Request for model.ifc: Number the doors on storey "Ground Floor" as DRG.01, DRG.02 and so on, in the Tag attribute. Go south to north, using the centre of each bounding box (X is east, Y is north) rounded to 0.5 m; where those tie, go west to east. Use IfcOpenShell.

First a look at what the model holds.

```python
import ifcopenshell
import ifcopenshell.util.element
import ifcopenshell.util.placement

model = ifcopenshell.open("model.ifc")
print(model.schema)
storey = next(s for s in model.by_type("IfcBuildingStorey") if s.Name == "Ground Floor")
doors = [e for e in ifcopenshell.util.element.get_decomposition(storey) if e.is_a("IfcDoor")]
for e in sorted(doors, key=lambda e: e.id()):
    origin = ifcopenshell.util.placement.get_local_placement(e.ObjectPlacement)[:3, 3]
    print(e.id(), e.Tag, e.Name, origin.round(2) + 0.0, sep=" | ")
```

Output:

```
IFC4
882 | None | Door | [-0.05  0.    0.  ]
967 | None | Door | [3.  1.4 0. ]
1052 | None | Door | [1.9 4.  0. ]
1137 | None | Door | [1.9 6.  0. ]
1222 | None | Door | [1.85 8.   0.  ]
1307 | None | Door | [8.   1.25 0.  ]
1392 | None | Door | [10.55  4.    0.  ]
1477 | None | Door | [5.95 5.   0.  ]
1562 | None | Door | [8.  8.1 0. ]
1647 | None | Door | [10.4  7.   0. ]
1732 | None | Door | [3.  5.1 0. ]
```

```python
import ifcopenshell
import ifcopenshell.geom
import ifcopenshell.util.element
import ifcopenshell.util.shape

model = ifcopenshell.open("model.ifc")
settings = ifcopenshell.geom.settings()
settings.set("use-world-coords", True)


def centre(element):
    shape = ifcopenshell.geom.create_shape(settings, element)
    return ifcopenshell.util.shape.get_bbox_centroid(shape.geometry)


storey = next(s for s in model.by_type("IfcBuildingStorey") if s.Name == "Ground Floor")
doors = [e for e in ifcopenshell.util.element.get_decomposition(storey) if e.is_a("IfcDoor")]

# Insertion points can sit at a corner or the storey origin, so sort by the geometry (in metres).
centres = {e: centre(e) for e in doors}
doors.sort(key=lambda e: (round(centres[e][1] / 0.5), centres[e][0]))

for i, e in enumerate(doors, start=1):
    number = f"DRG.{i:02d}"
    e.Tag = number
    print(e.id(), number)

model.write("model_v2.ifc")
```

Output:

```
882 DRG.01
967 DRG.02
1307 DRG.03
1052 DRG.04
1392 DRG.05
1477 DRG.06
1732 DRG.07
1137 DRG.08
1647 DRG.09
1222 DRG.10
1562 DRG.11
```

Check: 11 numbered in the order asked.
